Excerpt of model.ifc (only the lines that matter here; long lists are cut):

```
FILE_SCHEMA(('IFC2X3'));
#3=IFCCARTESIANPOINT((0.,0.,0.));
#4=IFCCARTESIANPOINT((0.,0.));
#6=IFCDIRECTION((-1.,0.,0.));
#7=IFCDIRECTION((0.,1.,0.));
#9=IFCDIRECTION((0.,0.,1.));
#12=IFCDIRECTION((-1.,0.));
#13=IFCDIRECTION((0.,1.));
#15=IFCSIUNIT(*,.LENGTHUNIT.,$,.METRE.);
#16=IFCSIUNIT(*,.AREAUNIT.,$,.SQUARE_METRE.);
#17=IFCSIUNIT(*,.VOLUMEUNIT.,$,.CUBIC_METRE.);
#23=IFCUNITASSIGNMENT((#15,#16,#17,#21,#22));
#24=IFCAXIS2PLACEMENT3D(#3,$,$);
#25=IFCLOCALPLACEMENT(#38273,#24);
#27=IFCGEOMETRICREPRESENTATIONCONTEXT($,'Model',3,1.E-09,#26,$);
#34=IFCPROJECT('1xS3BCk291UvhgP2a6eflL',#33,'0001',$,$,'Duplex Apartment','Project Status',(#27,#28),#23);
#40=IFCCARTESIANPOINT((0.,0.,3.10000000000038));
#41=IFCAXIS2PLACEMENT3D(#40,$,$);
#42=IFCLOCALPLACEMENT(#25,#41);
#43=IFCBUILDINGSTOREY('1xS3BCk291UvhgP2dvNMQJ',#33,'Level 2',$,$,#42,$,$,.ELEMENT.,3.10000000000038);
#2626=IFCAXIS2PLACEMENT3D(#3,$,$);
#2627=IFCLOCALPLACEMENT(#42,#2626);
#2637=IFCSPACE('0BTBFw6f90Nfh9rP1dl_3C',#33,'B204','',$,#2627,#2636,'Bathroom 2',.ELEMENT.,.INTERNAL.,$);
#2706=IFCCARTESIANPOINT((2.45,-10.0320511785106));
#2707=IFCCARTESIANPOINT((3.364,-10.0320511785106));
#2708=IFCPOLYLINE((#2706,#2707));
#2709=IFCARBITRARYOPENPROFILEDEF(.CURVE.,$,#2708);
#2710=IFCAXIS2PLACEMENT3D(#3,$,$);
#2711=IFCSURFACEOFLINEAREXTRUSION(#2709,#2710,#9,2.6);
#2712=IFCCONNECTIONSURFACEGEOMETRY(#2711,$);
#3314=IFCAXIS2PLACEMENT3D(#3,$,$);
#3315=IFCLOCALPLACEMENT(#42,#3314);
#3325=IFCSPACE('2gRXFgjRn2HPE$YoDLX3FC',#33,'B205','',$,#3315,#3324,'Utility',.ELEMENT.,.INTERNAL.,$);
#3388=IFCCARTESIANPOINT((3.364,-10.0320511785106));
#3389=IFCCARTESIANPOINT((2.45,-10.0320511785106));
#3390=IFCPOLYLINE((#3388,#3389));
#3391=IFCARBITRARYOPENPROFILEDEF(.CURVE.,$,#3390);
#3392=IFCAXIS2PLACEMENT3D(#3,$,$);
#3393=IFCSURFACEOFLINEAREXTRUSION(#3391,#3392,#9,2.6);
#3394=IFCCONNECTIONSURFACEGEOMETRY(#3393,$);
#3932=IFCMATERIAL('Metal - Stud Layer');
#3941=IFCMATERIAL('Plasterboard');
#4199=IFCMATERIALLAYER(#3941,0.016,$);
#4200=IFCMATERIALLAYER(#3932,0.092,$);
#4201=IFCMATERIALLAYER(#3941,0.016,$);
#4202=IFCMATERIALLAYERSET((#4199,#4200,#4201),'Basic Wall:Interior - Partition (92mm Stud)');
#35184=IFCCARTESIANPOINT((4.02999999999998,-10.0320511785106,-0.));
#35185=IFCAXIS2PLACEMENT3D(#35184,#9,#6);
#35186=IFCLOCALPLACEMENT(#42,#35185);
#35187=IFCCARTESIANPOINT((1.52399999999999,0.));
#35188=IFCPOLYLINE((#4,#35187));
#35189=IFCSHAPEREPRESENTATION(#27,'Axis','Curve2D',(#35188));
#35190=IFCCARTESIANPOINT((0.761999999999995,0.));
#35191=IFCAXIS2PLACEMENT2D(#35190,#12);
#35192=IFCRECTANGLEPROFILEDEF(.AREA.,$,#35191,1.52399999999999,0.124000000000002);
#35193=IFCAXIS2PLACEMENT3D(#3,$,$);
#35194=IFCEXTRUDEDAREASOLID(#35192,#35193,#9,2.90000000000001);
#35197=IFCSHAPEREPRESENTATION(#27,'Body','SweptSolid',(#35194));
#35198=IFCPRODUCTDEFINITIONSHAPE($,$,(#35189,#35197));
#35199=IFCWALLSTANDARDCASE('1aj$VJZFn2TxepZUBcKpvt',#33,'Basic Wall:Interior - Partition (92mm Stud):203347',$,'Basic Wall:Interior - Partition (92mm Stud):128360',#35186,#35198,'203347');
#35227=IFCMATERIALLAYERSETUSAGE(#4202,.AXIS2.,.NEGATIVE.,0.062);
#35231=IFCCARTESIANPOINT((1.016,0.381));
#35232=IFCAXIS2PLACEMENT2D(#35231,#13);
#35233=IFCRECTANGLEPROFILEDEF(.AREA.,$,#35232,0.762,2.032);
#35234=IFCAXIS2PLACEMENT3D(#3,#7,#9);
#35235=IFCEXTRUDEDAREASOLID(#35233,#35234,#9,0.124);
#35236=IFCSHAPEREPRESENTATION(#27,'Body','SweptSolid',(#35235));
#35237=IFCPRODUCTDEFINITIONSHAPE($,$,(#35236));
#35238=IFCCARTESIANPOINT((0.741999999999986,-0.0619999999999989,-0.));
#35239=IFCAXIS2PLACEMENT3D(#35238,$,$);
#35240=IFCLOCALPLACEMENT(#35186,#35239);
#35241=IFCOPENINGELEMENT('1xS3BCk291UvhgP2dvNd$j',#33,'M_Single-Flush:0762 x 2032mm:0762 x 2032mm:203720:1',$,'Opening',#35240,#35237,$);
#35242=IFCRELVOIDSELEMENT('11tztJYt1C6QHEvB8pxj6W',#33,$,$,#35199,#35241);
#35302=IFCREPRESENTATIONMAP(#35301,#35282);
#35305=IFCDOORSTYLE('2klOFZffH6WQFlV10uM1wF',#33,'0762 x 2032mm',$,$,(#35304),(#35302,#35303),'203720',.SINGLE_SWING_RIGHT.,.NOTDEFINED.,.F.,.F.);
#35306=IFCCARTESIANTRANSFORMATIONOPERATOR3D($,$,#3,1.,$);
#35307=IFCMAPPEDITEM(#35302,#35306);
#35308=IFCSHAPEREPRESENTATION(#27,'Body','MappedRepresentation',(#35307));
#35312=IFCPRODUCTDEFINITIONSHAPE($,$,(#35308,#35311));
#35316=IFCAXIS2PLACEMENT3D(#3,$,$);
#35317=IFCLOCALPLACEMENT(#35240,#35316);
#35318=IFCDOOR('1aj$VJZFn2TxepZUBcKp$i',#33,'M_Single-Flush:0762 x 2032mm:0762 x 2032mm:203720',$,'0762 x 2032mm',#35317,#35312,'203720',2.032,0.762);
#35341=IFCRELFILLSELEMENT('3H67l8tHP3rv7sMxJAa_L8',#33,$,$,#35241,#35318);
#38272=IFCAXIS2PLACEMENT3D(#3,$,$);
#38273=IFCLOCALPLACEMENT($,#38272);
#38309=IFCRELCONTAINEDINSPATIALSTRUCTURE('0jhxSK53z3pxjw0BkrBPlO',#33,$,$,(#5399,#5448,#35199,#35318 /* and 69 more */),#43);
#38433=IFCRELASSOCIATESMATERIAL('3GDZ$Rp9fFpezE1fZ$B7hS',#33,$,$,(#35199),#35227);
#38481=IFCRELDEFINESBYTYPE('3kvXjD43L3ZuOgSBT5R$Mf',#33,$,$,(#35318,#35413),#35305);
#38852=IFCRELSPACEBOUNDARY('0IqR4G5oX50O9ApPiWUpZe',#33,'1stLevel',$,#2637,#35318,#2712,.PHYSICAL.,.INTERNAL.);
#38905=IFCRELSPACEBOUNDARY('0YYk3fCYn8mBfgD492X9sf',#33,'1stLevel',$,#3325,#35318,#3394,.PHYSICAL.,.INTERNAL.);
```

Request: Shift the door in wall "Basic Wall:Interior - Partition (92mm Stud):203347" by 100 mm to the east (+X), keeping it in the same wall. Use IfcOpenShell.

```python
import numpy as np
import ifcopenshell
import ifcopenshell.api.geometry
import ifcopenshell.util.placement
import ifcopenshell.util.unit

model = ifcopenshell.open("model.ifc")
unit_scale = ifcopenshell.util.unit.calculate_unit_scale(model)

door = model.by_guid("1aj$VJZFn2TxepZUBcKp$i")
opening = door.FillsVoids[0].RelatingOpeningElement
wall = opening.VoidsElements[0].RelatingBuildingElement

wall_matrix = ifcopenshell.util.placement.get_local_placement(wall.ObjectPlacement)
shift = wall_matrix[:3, 0] * -0.1 / unit_scale
before = ifcopenshell.util.placement.get_local_placement(door.ObjectPlacement)[:3, 3].copy()

# The door is placed relative to its opening, so it follows when the opening moves.
matrix = ifcopenshell.util.placement.get_local_placement(opening.ObjectPlacement)
matrix[:3, 3] += shift
ifcopenshell.api.geometry.edit_object_placement(
    model, product=opening, matrix=matrix, is_si=False, should_transform_children=True
)

# Space boundary surfaces are stored in each space's coordinates; move them too.
for rel in door.ProvidesBoundaries:
    if not rel.ConnectionGeometry:
        continue
    surface = rel.ConnectionGeometry.SurfaceOnRelatingElement
    space_matrix = ifcopenshell.util.placement.get_local_placement(rel.RelatingSpace.ObjectPlacement)
    point = np.array(surface.Position.Location.Coordinates) + space_matrix[:3, :3].T @ shift
    surface.Position = model.createIfcAxis2Placement3D(
        model.createIfcCartesianPoint(point.tolist()), surface.Position.Axis, surface.Position.RefDirection
    )

after = ifcopenshell.util.placement.get_local_placement(door.ObjectPlacement)[:3, 3]
print("door moved by", (after - before).round(3) + 0.0)

model.write("model_rev.ifc")
```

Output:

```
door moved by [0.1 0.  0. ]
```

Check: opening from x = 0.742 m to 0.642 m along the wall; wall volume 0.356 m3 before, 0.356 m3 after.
